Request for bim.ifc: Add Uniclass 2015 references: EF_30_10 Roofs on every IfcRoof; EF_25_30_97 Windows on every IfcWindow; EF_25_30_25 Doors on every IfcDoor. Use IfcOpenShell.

First a look at what the model holds.

```python
import ifcopenshell

model = ifcopenshell.open("bim.ifc")
print(model.schema)
print("classifications:", [c.Name for c in model.by_type("IfcClassification")])
for ifc_class in ("IfcDoor", "IfcRoof", "IfcStair", "IfcWall", "IfcWindow"):
    print(ifc_class, len(model.by_type(ifc_class)))
```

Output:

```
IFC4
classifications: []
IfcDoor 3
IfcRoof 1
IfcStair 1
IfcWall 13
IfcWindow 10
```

```python
import ifcopenshell
import ifcopenshell.api.classification

model = ifcopenshell.open("bim.ifc")

system = ifcopenshell.api.classification.add_classification(model, classification="Uniclass 2015")

codes = {
    "IfcRoof": ("EF_30_10", "Roofs"),
    "IfcWindow": ("EF_25_30_97", "Windows"),
    "IfcDoor": ("EF_25_30_25", "Doors"),
}
for ifc_class, (code, name) in codes.items():
    products = model.by_type(ifc_class)
    ifcopenshell.api.classification.add_reference(
        model, products=products, classification=system, identification=code, name=name
    )
    print(code, len(products))

model.write("bim_v2.ifc")
```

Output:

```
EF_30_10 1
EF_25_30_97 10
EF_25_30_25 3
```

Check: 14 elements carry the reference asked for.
